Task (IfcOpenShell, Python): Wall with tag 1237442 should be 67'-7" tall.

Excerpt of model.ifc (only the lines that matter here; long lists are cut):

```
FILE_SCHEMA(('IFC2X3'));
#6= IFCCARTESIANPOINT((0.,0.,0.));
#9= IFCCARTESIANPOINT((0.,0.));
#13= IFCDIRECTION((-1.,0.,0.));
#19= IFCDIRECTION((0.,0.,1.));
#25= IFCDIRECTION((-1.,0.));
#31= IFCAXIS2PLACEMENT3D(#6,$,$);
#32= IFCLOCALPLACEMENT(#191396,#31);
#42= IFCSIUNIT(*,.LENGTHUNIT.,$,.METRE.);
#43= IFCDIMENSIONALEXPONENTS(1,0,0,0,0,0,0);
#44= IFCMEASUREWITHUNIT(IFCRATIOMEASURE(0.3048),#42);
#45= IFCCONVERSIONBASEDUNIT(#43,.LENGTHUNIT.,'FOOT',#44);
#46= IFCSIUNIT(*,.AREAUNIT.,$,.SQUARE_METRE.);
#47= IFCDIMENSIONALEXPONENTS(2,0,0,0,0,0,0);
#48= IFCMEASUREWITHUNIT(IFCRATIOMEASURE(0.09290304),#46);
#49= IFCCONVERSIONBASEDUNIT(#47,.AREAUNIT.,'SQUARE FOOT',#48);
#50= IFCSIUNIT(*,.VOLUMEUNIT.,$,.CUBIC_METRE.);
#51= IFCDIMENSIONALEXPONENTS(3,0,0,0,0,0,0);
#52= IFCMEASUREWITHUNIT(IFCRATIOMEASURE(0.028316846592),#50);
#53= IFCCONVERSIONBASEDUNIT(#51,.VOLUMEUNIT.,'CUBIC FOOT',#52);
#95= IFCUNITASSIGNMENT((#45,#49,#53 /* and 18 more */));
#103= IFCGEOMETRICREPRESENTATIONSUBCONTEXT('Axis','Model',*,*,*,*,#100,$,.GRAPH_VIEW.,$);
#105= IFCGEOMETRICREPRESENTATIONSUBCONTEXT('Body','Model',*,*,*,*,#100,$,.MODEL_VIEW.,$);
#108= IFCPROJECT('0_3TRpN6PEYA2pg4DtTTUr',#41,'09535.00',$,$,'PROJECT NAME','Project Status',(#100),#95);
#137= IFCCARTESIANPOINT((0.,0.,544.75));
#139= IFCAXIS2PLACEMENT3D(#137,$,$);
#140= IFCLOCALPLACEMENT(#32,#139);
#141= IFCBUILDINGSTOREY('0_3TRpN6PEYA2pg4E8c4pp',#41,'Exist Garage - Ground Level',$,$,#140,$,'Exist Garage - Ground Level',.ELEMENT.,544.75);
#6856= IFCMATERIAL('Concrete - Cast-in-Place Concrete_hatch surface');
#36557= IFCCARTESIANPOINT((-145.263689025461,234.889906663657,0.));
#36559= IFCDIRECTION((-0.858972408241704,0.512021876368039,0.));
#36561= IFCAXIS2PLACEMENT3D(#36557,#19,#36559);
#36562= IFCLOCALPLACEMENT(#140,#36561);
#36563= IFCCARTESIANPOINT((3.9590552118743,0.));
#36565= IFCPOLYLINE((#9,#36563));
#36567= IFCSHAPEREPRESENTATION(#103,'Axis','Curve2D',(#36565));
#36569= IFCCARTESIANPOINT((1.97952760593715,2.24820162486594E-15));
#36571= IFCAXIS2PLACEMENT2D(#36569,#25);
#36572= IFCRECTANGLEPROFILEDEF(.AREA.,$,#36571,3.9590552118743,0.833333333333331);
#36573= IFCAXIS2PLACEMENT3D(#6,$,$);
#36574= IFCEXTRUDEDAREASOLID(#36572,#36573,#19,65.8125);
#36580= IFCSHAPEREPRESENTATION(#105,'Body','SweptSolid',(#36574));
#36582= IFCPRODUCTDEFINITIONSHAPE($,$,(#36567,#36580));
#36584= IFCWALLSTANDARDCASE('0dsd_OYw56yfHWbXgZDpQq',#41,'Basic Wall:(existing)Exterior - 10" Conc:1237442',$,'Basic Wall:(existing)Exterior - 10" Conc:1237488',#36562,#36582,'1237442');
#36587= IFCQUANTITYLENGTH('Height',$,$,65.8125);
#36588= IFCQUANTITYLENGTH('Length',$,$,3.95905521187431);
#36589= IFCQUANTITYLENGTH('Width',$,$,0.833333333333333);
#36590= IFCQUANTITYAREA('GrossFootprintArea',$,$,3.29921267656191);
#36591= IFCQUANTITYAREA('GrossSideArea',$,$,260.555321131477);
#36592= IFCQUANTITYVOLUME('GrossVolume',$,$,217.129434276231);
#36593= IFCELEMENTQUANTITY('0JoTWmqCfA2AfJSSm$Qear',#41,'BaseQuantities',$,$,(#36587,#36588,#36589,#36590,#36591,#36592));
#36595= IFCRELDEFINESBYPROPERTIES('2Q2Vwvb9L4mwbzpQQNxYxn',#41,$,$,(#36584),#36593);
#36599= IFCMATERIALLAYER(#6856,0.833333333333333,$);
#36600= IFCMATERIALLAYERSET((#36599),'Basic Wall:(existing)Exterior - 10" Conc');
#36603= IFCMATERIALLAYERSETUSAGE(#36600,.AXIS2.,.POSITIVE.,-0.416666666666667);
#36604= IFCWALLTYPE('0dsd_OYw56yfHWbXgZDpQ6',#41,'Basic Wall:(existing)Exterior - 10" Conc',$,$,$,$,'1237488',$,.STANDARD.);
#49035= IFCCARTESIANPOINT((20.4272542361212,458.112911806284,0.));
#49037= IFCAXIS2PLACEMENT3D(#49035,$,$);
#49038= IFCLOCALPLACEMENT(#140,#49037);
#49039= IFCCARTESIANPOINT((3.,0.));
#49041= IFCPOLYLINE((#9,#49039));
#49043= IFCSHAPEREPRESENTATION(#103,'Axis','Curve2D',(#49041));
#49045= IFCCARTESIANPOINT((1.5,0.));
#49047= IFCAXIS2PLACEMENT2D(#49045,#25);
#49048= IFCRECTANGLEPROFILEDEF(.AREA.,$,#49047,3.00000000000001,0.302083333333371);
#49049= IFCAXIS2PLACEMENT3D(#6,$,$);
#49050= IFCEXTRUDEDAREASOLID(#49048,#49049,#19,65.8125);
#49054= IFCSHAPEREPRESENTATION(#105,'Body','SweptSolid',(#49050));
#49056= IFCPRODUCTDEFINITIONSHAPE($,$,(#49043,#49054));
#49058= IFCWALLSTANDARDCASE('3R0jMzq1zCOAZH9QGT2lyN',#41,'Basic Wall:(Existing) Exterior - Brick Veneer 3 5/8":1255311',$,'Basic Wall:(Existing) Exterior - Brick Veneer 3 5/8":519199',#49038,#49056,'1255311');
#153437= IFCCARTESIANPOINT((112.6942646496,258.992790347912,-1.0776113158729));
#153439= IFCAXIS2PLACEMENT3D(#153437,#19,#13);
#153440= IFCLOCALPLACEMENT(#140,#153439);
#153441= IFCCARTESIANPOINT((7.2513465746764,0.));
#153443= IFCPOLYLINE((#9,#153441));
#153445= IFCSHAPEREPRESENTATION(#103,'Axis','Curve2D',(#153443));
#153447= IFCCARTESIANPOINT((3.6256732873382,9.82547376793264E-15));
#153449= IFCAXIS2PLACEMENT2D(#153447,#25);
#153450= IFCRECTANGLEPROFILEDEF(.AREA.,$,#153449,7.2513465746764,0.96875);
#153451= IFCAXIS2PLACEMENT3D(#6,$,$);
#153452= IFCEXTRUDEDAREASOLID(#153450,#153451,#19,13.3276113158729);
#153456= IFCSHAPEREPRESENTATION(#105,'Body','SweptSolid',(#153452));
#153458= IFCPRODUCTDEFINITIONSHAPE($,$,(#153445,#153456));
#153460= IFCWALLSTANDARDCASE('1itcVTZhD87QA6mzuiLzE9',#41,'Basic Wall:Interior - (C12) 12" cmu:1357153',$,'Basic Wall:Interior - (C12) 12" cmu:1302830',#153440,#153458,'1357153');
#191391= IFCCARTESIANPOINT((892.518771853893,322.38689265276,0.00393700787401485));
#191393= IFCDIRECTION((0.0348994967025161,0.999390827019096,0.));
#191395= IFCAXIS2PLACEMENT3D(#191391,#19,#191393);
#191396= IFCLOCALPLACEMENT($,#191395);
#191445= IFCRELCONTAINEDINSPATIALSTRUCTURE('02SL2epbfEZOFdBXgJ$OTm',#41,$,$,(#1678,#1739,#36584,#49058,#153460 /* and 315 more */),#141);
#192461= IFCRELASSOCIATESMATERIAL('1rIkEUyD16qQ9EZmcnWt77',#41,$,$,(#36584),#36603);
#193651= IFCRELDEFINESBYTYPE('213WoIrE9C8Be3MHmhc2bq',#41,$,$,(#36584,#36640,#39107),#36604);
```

```python
import ifcopenshell
import ifcopenshell.api.pset
import ifcopenshell.geom
import ifcopenshell.util.element
import ifcopenshell.util.representation
import ifcopenshell.util.shape
import ifcopenshell.util.unit

model = ifcopenshell.open("model.ifc")
unit_scale = ifcopenshell.util.unit.calculate_unit_scale(model)
area_scale = ifcopenshell.util.unit.calculate_unit_scale(model, "AREAUNIT")
volume_scale = ifcopenshell.util.unit.calculate_unit_scale(model, "VOLUMEUNIT")
settings = ifcopenshell.geom.settings()


def volume(element):
    """Net volume in cubic metres, openings subtracted."""
    shape = ifcopenshell.geom.create_shape(settings, element)
    return ifcopenshell.util.shape.get_volume(shape.geometry)


wall = model.by_id(36584)
before = volume(wall)

body = ifcopenshell.util.representation.get_representation(wall, "Model", "Body")
solid = body.Items[0]
old_height = solid.Depth
solid.Depth = 811 * 0.0254 / unit_scale
after = volume(wall)

# Update the stored height, areas and volumes.
qto = model.by_id(ifcopenshell.util.element.get_pset(wall, "BaseQuantities", should_inherit=False)["id"])
ifcopenshell.api.pset.edit_qto(model, qto=qto, properties={
    "Height": solid.Depth,
    "GrossSideArea": ifcopenshell.util.element.get_pset(wall, "BaseQuantities", "GrossSideArea") * solid.Depth / old_height,
    "GrossVolume": ifcopenshell.util.element.get_pset(wall, "BaseQuantities", "GrossVolume") * solid.Depth / old_height,
})

print(f"height {old_height:g} -> {solid.Depth:g}, volume {before:.3f} -> {after:.3f} m3")

model.write("model_v2.ifc")
```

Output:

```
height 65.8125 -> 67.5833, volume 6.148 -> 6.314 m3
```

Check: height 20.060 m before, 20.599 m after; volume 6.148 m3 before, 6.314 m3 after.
